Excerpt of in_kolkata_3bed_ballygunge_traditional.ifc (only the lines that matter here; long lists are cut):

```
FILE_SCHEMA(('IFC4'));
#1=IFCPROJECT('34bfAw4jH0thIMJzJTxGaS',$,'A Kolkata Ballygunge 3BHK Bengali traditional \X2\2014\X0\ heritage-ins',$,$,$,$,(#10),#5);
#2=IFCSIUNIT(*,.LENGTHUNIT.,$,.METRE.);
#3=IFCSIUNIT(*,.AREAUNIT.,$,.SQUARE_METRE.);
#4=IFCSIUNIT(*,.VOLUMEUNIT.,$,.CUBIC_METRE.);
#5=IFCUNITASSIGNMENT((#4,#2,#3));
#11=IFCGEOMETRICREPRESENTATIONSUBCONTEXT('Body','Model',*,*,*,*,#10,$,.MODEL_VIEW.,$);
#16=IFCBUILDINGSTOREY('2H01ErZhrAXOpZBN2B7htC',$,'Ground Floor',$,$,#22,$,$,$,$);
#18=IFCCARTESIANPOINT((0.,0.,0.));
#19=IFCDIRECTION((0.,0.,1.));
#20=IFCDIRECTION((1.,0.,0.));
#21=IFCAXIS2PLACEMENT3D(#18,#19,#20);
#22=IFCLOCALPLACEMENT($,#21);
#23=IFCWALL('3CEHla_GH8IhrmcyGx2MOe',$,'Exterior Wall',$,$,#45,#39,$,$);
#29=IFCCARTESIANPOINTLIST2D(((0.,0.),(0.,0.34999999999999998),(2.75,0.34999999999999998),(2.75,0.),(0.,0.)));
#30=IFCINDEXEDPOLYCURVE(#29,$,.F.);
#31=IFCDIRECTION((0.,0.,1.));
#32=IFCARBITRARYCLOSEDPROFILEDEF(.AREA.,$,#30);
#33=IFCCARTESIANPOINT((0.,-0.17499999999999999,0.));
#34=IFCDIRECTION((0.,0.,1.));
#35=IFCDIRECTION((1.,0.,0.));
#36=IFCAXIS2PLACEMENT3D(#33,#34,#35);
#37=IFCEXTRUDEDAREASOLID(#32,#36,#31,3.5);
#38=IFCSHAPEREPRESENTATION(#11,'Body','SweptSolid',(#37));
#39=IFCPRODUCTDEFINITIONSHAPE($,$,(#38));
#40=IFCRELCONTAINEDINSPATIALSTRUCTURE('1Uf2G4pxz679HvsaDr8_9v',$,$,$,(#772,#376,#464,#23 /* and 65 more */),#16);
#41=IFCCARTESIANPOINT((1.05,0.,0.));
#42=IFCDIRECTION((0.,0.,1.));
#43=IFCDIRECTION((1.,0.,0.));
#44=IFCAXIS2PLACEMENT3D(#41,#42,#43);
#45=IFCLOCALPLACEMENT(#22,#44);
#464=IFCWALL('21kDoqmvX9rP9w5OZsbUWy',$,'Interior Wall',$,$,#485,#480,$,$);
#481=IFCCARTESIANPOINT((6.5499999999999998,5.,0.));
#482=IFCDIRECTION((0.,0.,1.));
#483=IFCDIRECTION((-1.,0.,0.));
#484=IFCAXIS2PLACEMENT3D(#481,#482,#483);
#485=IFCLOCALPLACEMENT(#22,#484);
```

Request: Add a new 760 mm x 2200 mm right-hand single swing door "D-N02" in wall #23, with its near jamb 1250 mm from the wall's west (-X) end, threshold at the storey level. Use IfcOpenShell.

```python
import numpy as np
import ifcopenshell
import ifcopenshell.api.feature
import ifcopenshell.api.geometry
import ifcopenshell.api.root
import ifcopenshell.api.spatial
import ifcopenshell.geom
import ifcopenshell.util.element
import ifcopenshell.util.placement
import ifcopenshell.util.representation
import ifcopenshell.util.shape
import ifcopenshell.util.unit

model = ifcopenshell.open("in_kolkata_3bed_ballygunge_traditional.ifc")
unit_scale = ifcopenshell.util.unit.calculate_unit_scale(model)
settings = ifcopenshell.geom.settings()


def volume(element):
    """Net volume in cubic metres, openings subtracted."""
    shape = ifcopenshell.geom.create_shape(settings, element)
    return ifcopenshell.util.shape.get_volume(shape.geometry)


wall = model.by_guid("3CEHla_GH8IhrmcyGx2MOe")
storey = ifcopenshell.util.element.get_container(wall, ifc_class="IfcBuildingStorey")
context = ifcopenshell.util.representation.get_context(model, "Model", "Body", "MODEL_VIEW")
before = volume(wall)

width, height, from_end, sill = 0.76, 2.2, 1.25, 0.0  # metres

# The wall runs along its own X axis, and the end named is its -X end.
wall_shape = ifcopenshell.geom.create_shape(settings, wall)
x, y, z = ifcopenshell.util.shape.get_vertices(wall_shape.geometry).T
start = x.min() + from_end
face, thickness = float(y.min()), float(y.max() - y.min())
wall_matrix = ifcopenshell.util.placement.get_local_placement(wall.ObjectPlacement)
level = ifcopenshell.util.placement.get_local_placement(storey.ObjectPlacement)[2, 3]


def in_wall(x, y):
    """Placement at x, y metres in the wall's axes, at sill height."""
    matrix = wall_matrix.copy()
    matrix[:, 3] = wall_matrix @ np.array([x / unit_scale, y / unit_scale, 0.0, 1.0])
    matrix[2, 3] = level + sill / unit_scale
    return matrix


# Opening: a box that overshoots both wall faces by 50 mm.
opening = ifcopenshell.api.root.create_entity(model, ifc_class="IfcOpeningElement", predefined_type="OPENING")
box = ifcopenshell.api.geometry.add_wall_representation(
    model, context=context, length=width, height=height, thickness=thickness + 0.1
)
ifcopenshell.api.geometry.assign_representation(model, product=opening, representation=box)
ifcopenshell.api.geometry.edit_object_placement(model, product=opening, matrix=in_wall(start, face - 0.05), is_si=False)
ifcopenshell.api.feature.add_feature(model, feature=opening, element=wall)

door = ifcopenshell.api.root.create_entity(model, ifc_class="IfcDoor", name="D-N02", predefined_type="DOOR")
door.OverallWidth, door.OverallHeight = width / unit_scale, height / unit_scale
door.OperationType = "SINGLE_SWING_RIGHT"
body = ifcopenshell.api.geometry.add_door_representation(
    model,
    context=context,
    overall_width=door.OverallWidth,
    overall_height=door.OverallHeight,
    operation_type="SINGLE_SWING_RIGHT",
    lining_properties={"LiningDepth": thickness / unit_scale, "ThresholdDepth": thickness / unit_scale},
)
ifcopenshell.api.geometry.assign_representation(model, product=door, representation=body)
ifcopenshell.api.spatial.assign_container(model, products=[door], relating_structure=storey)
ifcopenshell.api.feature.add_filling(model, opening=opening, element=door)

# The lining spans the wall, so the door starts at the wall face.
ifcopenshell.api.geometry.edit_object_placement(model, product=door, matrix=in_wall(start, face), is_si=False)

after = volume(wall)

print(f"wall volume {before:.3f} -> {after:.3f} m3")

model.write("in_kolkata_3bed_ballygunge_traditional_edited.ifc")
```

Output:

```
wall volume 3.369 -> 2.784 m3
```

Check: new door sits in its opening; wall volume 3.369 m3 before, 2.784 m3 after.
